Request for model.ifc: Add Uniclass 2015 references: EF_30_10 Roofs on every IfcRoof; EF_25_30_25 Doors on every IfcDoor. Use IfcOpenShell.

First a look at what the model holds.

```python
import ifcopenshell

model = ifcopenshell.open("model.ifc")
print(model.schema)
print("classifications:", [c.Name for c in model.by_type("IfcClassification")])
for ifc_class in ("IfcDoor", "IfcRoof", "IfcStair", "IfcWall", "IfcWindow"):
    print(ifc_class, len(model.by_type(ifc_class)))
```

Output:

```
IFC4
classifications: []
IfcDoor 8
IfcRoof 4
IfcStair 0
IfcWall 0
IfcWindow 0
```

```python
import ifcopenshell
import ifcopenshell.api.classification

model = ifcopenshell.open("model.ifc")

system = ifcopenshell.api.classification.add_classification(model, classification="Uniclass 2015")

codes = {
    "IfcRoof": ("EF_30_10", "Roofs"),
    "IfcDoor": ("EF_25_30_25", "Doors"),
}
for ifc_class, (code, name) in codes.items():
    products = model.by_type(ifc_class)
    ifcopenshell.api.classification.add_reference(
        model, products=products, classification=system, identification=code, name=name
    )
    print(code, len(products))

model.write("model_updated.ifc")
```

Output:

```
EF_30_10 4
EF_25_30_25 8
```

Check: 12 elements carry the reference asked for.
